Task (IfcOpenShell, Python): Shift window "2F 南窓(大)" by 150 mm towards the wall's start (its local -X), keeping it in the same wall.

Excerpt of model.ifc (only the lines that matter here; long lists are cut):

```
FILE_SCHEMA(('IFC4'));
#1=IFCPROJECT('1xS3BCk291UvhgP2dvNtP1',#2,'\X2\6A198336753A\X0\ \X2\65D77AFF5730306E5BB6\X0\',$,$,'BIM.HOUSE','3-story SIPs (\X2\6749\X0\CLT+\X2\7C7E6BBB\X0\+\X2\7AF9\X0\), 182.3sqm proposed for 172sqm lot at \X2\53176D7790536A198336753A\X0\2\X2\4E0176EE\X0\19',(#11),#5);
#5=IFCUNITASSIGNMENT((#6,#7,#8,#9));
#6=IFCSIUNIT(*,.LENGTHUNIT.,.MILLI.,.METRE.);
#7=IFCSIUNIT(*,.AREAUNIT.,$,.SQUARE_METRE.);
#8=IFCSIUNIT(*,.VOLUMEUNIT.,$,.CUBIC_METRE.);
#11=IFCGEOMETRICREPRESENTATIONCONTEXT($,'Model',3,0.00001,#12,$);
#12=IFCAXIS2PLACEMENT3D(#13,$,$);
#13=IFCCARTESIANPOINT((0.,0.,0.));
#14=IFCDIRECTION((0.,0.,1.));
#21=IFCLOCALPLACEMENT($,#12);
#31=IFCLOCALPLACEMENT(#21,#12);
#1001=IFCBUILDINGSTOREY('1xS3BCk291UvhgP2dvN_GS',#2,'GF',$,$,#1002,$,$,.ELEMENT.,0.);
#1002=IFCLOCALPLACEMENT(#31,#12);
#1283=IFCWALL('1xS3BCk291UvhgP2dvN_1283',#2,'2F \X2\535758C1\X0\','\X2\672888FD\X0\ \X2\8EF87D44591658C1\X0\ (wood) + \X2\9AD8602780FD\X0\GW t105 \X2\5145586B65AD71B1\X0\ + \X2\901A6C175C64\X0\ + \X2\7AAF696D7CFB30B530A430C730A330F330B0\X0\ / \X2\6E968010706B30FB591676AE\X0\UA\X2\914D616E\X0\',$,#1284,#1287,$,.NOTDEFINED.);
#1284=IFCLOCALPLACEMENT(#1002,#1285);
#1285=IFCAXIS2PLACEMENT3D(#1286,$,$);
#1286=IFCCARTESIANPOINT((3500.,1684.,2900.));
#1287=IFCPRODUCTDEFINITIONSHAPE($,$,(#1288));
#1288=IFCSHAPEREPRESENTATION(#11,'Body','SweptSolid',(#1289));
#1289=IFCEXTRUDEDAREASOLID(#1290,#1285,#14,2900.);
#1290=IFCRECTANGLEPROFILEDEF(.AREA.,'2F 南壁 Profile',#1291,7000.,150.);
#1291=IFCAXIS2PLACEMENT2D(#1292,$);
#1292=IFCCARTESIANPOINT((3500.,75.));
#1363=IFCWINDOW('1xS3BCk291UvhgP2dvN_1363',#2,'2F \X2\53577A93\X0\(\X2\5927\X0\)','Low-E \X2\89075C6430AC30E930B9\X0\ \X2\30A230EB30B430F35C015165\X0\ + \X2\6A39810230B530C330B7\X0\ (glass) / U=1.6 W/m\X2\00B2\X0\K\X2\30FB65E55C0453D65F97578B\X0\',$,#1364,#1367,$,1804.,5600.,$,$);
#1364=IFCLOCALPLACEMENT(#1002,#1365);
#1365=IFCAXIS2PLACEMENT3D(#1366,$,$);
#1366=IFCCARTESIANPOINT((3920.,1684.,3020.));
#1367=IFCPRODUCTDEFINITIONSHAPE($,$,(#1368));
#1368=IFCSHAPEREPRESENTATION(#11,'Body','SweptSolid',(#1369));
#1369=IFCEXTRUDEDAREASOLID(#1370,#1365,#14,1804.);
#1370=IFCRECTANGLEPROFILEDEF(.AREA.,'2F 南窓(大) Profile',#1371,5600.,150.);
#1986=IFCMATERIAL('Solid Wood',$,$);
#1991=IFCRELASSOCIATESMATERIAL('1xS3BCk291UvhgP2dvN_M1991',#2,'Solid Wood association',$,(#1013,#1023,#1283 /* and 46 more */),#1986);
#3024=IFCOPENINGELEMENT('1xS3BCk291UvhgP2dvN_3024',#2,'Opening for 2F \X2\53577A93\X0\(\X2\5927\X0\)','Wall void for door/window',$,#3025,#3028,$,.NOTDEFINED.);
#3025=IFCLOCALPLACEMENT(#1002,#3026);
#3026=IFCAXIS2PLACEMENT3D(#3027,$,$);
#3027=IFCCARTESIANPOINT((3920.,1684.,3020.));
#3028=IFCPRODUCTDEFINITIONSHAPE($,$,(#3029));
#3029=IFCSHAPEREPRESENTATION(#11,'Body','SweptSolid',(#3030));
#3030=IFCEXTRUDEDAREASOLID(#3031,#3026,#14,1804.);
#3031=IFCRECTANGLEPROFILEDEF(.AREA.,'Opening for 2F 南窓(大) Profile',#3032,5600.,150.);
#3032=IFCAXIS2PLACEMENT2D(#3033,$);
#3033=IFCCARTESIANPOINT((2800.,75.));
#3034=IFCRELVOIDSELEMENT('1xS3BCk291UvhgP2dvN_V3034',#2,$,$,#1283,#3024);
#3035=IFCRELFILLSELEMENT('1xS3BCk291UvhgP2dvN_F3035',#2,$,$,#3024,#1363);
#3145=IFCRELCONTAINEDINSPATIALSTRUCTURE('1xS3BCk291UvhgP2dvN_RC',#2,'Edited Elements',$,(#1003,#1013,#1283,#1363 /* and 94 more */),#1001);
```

```python
import ifcopenshell
import ifcopenshell.api.geometry
import ifcopenshell.util.placement
import ifcopenshell.util.unit

model = ifcopenshell.open("model.ifc")
unit_scale = ifcopenshell.util.unit.calculate_unit_scale(model)

window = model.by_guid("1xS3BCk291UvhgP2dvN_1363")
opening = window.FillsVoids[0].RelatingOpeningElement
wall = opening.VoidsElements[0].RelatingBuildingElement

wall_matrix = ifcopenshell.util.placement.get_local_placement(wall.ObjectPlacement)
shift = wall_matrix[:3, 0] * -0.15 / unit_scale
before = ifcopenshell.util.placement.get_local_placement(window.ObjectPlacement)[:3, 3].copy()

# The window is not placed relative to its opening, so move both.
for product in (opening, window):
    matrix = ifcopenshell.util.placement.get_local_placement(product.ObjectPlacement)
    matrix[:3, 3] += shift
    ifcopenshell.api.geometry.edit_object_placement(model, product=product, matrix=matrix, is_si=False)

after = ifcopenshell.util.placement.get_local_placement(window.ObjectPlacement)[:3, 3]
print("window moved by", (after - before).round(3) + 0.0)

model.write("model_edited.ifc")
```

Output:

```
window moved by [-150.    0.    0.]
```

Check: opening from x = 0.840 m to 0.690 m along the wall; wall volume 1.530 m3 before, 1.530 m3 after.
